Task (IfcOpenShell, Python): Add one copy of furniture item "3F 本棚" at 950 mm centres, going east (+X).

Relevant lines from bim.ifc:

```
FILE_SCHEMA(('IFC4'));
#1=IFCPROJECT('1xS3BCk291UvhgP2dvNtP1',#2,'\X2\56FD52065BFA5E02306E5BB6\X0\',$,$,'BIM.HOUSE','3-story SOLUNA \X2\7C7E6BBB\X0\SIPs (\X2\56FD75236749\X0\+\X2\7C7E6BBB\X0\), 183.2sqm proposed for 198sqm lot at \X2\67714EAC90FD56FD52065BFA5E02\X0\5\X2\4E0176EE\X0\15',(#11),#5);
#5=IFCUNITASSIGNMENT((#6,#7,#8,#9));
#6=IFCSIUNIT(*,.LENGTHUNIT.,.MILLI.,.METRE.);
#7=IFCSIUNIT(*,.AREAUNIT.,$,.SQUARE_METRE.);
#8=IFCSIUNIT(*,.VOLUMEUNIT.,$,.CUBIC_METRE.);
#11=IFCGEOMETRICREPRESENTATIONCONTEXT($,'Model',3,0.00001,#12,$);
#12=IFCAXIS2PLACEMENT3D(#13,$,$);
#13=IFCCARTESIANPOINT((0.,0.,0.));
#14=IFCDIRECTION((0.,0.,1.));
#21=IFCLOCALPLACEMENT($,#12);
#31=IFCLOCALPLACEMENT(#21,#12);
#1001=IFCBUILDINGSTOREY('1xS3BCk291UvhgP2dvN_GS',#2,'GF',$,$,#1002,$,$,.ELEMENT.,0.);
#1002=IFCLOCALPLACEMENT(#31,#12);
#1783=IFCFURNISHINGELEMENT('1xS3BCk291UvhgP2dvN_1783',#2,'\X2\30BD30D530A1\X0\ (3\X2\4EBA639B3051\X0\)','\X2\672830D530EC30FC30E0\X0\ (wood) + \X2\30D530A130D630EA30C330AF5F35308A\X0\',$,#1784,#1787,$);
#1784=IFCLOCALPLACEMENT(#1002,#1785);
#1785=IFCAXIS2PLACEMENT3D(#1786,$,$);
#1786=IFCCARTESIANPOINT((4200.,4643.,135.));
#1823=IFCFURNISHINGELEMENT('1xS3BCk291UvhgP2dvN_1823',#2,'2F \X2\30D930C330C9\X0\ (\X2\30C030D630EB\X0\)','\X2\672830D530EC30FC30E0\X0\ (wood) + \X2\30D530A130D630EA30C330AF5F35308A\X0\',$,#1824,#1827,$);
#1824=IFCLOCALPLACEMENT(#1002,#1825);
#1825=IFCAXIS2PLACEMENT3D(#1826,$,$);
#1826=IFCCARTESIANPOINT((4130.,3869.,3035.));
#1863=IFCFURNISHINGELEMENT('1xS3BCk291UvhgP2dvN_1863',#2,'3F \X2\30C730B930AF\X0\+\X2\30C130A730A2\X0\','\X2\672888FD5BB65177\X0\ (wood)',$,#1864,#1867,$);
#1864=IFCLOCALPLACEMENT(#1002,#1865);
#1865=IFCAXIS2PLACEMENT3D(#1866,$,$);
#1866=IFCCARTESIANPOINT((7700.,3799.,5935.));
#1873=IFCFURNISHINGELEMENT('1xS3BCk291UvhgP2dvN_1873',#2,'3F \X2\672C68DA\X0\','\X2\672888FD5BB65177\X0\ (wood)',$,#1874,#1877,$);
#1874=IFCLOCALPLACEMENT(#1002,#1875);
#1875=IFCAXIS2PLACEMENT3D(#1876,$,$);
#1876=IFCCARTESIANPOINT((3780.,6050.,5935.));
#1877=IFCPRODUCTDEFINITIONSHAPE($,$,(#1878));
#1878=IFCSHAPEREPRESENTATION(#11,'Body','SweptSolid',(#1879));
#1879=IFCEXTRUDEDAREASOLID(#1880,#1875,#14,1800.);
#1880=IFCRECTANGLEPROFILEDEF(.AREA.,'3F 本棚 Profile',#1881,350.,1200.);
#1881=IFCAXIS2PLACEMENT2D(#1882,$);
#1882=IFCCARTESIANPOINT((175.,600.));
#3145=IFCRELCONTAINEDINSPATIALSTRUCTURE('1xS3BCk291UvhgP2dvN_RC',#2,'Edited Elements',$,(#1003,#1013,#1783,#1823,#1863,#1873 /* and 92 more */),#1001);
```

```python
import numpy as np
import ifcopenshell
import ifcopenshell.api.geometry
import ifcopenshell.api.root
import ifcopenshell.util.element
import ifcopenshell.util.placement
import ifcopenshell.util.unit

model = ifcopenshell.open("bim.ifc")
unit_scale = ifcopenshell.util.unit.calculate_unit_scale(model)


def reuse_history(source, copy):
    """copy_class also copies each property set's owner history, people and application; keep the originals."""
    for rel in copy.IsDefinedBy:
        if rel.is_a("IfcRelDefinesByProperties") and (history := rel.RelatingPropertyDefinition.OwnerHistory):
            rel.RelatingPropertyDefinition.OwnerHistory = source.OwnerHistory
            ifcopenshell.util.element.remove_deep2(model, history)


source = model.by_guid("1xS3BCk291UvhgP2dvN_1873")
base = ifcopenshell.util.placement.get_local_placement(source.ObjectPlacement)
step = np.array([1.0, 0.0, 0.0]) * 0.95 / unit_scale

for i in range(1, 2):
    copy = ifcopenshell.api.root.copy_class(model, product=source)
    copy.Representation = ifcopenshell.util.element.copy_deep(
        model, source.Representation, exclude=["IfcGeometricRepresentationContext", "IfcRepresentationMap"]
    )
    reuse_history(source, copy)
    matrix = base.copy()
    matrix[:3, 3] += i * step
    print("added at", matrix[:3, 3].round(3) + 0.0)
    ifcopenshell.api.geometry.edit_object_placement(model, product=copy, matrix=matrix, is_si=False)

model.write("bim_rev.ifc")
```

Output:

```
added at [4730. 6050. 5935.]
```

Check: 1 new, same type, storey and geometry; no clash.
